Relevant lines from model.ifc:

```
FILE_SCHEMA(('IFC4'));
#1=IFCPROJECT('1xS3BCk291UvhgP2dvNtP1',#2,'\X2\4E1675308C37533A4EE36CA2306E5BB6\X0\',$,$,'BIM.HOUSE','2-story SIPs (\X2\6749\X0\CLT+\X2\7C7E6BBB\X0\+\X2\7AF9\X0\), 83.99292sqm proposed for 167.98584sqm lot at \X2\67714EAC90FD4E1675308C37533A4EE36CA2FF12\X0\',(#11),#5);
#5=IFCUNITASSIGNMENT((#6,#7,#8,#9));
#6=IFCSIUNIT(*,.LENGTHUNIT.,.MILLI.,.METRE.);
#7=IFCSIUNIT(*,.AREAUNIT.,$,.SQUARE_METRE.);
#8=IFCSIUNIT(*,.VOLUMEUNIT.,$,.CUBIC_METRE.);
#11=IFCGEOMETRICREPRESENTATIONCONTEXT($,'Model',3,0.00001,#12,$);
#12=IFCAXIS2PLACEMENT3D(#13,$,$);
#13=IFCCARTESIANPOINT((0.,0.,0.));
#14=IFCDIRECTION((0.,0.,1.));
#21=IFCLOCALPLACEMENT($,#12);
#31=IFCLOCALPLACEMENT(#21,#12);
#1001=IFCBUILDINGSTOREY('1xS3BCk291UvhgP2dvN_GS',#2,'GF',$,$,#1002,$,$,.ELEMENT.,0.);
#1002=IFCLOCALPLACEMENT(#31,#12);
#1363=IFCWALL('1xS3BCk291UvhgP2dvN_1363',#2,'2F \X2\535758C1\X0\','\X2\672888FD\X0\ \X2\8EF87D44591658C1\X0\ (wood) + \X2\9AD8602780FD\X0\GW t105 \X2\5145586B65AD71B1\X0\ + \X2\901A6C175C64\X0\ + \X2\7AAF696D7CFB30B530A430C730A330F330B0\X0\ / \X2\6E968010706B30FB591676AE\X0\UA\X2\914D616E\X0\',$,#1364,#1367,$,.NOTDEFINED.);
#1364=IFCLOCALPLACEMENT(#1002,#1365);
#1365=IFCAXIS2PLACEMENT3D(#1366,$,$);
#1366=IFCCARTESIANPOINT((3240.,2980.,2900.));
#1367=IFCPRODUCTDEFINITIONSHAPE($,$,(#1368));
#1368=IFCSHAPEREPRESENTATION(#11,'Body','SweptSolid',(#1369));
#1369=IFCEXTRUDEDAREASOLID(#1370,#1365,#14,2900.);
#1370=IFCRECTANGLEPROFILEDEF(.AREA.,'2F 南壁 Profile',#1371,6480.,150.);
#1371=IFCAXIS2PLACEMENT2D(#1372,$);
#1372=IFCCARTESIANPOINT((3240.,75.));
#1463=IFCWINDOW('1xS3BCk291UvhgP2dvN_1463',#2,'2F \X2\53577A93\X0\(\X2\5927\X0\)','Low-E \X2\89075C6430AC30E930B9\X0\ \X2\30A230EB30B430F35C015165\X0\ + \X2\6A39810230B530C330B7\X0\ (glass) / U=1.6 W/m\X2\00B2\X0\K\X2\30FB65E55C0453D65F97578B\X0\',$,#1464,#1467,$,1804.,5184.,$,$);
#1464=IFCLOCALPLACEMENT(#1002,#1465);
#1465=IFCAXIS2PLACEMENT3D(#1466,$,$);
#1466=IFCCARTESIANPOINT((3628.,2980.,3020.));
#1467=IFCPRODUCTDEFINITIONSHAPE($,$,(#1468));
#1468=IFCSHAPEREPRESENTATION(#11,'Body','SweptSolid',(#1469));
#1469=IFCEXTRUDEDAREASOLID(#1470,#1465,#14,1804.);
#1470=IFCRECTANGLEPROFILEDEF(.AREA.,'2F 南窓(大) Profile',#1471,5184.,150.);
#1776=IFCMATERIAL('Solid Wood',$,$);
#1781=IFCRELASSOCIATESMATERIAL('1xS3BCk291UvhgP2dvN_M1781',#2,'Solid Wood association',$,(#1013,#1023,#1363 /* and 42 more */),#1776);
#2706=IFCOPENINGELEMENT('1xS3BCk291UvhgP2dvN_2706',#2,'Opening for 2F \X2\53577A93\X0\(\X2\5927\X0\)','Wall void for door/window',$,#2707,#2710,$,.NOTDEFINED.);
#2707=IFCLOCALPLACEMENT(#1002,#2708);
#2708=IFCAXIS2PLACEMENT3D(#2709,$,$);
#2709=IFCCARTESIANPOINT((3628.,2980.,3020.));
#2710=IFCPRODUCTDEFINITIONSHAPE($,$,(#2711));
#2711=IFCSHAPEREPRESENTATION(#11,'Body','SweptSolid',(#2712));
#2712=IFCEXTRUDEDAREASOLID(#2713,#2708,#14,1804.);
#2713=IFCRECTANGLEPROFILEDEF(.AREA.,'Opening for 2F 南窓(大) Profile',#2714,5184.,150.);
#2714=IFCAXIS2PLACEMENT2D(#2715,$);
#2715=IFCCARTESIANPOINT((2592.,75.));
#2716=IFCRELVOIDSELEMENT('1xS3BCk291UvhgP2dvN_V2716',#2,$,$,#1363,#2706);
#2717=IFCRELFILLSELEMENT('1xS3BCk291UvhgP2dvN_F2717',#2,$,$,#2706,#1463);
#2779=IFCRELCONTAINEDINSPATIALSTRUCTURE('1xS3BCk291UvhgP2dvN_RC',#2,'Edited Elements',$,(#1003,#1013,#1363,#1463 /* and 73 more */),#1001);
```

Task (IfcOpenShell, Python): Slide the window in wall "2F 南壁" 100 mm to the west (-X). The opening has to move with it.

```python
import ifcopenshell
import ifcopenshell.api.geometry
import ifcopenshell.util.placement
import ifcopenshell.util.unit

model = ifcopenshell.open("model.ifc")
unit_scale = ifcopenshell.util.unit.calculate_unit_scale(model)

window = model.by_guid("1xS3BCk291UvhgP2dvN_1463")
opening = window.FillsVoids[0].RelatingOpeningElement
wall = opening.VoidsElements[0].RelatingBuildingElement

wall_matrix = ifcopenshell.util.placement.get_local_placement(wall.ObjectPlacement)
shift = wall_matrix[:3, 0] * -0.1 / unit_scale
before = ifcopenshell.util.placement.get_local_placement(window.ObjectPlacement)[:3, 3].copy()

# The window is not placed relative to its opening, so move both.
for product in (opening, window):
    matrix = ifcopenshell.util.placement.get_local_placement(product.ObjectPlacement)
    matrix[:3, 3] += shift
    ifcopenshell.api.geometry.edit_object_placement(model, product=product, matrix=matrix, is_si=False)

after = ifcopenshell.util.placement.get_local_placement(window.ObjectPlacement)[:3, 3]
print("window moved by", (after - before).round(3) + 0.0)

model.write("model_edited.ifc")
```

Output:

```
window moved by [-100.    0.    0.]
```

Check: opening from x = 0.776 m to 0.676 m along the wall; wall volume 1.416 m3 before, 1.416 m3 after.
